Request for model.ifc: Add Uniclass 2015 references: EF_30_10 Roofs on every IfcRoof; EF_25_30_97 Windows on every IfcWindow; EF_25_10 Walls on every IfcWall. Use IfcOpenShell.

First a look at what the model holds.

```python
import ifcopenshell

model = ifcopenshell.open("model.ifc")
print(model.schema)
print("classifications:", [c.Name for c in model.by_type("IfcClassification")])
for ifc_class in ("IfcDoor", "IfcRoof", "IfcStair", "IfcWall", "IfcWindow"):
    print(ifc_class, len(model.by_type(ifc_class)))
```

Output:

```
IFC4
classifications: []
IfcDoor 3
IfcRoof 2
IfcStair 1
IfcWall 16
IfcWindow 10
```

```python
import ifcopenshell
import ifcopenshell.api.classification

model = ifcopenshell.open("model.ifc")

system = ifcopenshell.api.classification.add_classification(model, classification="Uniclass 2015")

codes = {
    "IfcRoof": ("EF_30_10", "Roofs"),
    "IfcWindow": ("EF_25_30_97", "Windows"),
    "IfcWall": ("EF_25_10", "Walls"),
}
for ifc_class, (code, name) in codes.items():
    products = model.by_type(ifc_class)
    ifcopenshell.api.classification.add_reference(
        model, products=products, classification=system, identification=code, name=name
    )
    print(code, len(products))

model.write("model_rev.ifc")
```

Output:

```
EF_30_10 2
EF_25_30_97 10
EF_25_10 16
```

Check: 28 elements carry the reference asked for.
